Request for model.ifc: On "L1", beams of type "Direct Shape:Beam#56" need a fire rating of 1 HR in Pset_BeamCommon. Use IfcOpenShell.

First a look at what the model holds.

```python
import ifcopenshell
import ifcopenshell.util.element

model = ifcopenshell.open("model.ifc")
print(model.schema)
storey = next(s for s in model.by_type("IfcBuildingStorey") if s.Name == "L1")
beams = [e for e in ifcopenshell.util.element.get_decomposition(storey) if e.is_a("IfcBeam")]
seen = {}
for e in beams:
    element_type = ifcopenshell.util.element.get_type(e)
    key = (element_type.Name if element_type != e and element_type else None, ifcopenshell.util.element.get_pset(e, "Pset_BeamCommon", "FireRating"))
    seen[key] = seen.get(key, 0) + 1
for (name, value), count in sorted(seen.items(), key=str):
    print(count, "x", name, "|", value)
```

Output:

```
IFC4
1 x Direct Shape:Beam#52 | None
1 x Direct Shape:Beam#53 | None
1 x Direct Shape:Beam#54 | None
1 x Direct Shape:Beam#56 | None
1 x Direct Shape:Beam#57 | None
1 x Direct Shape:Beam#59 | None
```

```python
import ifcopenshell
import ifcopenshell.api.pset
import ifcopenshell.util.element

model = ifcopenshell.open("model.ifc")

storey = next(s for s in model.by_type("IfcBuildingStorey") if s.Name == "L1")
beams = [e for e in ifcopenshell.util.element.get_decomposition(storey) if e.is_a("IfcBeam")]

count = 0
for e in beams:
    element_type = ifcopenshell.util.element.get_type(e)
    if element_type in (None, e) or element_type.Name != "Direct Shape:Beam#56":
        continue
    # add_pset returns the element's existing set when there is one.
    pset = ifcopenshell.api.pset.add_pset(model, product=e, name="Pset_BeamCommon")
    ifcopenshell.api.pset.edit_pset(model, pset=pset, properties={"FireRating": "1 HR"})
    count += 1

print(count, "beams updated")

model.write("model_edited.ifc")
```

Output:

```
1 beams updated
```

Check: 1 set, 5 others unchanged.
